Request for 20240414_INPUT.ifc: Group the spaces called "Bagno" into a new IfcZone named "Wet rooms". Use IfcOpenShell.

First a look at what the model holds.

```python
import ifcopenshell

model = ifcopenshell.open("20240414_INPUT.ifc")
print(model.schema)
seen = {}
for space in model.by_type("IfcSpace"):
    seen[space.LongName] = seen.get(space.LongName, 0) + 1
for name, count in sorted(seen.items(), key=str):
    print(count, "x", name)
print("zones:", [z.Name for z in model.by_type("IfcZone")][:20])
```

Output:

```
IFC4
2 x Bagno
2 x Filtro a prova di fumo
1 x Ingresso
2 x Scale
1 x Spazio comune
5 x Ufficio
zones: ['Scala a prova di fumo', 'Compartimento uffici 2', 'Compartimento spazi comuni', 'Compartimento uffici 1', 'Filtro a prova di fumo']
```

```python
import ifcopenshell
import ifcopenshell.api.group
import ifcopenshell.api.root

model = ifcopenshell.open("20240414_INPUT.ifc")

names = {"Bagno"}
spaces = [s for s in model.by_type("IfcSpace") if s.LongName in names]

zone = ifcopenshell.api.root.create_entity(model, ifc_class="IfcZone", name="Wet rooms")
ifcopenshell.api.group.assign_group(model, products=spaces, group=zone)
print(len(spaces), "spaces in", zone.Name)

model.write("20240414_INPUT_edited.ifc")
```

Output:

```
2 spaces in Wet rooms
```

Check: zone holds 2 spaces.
